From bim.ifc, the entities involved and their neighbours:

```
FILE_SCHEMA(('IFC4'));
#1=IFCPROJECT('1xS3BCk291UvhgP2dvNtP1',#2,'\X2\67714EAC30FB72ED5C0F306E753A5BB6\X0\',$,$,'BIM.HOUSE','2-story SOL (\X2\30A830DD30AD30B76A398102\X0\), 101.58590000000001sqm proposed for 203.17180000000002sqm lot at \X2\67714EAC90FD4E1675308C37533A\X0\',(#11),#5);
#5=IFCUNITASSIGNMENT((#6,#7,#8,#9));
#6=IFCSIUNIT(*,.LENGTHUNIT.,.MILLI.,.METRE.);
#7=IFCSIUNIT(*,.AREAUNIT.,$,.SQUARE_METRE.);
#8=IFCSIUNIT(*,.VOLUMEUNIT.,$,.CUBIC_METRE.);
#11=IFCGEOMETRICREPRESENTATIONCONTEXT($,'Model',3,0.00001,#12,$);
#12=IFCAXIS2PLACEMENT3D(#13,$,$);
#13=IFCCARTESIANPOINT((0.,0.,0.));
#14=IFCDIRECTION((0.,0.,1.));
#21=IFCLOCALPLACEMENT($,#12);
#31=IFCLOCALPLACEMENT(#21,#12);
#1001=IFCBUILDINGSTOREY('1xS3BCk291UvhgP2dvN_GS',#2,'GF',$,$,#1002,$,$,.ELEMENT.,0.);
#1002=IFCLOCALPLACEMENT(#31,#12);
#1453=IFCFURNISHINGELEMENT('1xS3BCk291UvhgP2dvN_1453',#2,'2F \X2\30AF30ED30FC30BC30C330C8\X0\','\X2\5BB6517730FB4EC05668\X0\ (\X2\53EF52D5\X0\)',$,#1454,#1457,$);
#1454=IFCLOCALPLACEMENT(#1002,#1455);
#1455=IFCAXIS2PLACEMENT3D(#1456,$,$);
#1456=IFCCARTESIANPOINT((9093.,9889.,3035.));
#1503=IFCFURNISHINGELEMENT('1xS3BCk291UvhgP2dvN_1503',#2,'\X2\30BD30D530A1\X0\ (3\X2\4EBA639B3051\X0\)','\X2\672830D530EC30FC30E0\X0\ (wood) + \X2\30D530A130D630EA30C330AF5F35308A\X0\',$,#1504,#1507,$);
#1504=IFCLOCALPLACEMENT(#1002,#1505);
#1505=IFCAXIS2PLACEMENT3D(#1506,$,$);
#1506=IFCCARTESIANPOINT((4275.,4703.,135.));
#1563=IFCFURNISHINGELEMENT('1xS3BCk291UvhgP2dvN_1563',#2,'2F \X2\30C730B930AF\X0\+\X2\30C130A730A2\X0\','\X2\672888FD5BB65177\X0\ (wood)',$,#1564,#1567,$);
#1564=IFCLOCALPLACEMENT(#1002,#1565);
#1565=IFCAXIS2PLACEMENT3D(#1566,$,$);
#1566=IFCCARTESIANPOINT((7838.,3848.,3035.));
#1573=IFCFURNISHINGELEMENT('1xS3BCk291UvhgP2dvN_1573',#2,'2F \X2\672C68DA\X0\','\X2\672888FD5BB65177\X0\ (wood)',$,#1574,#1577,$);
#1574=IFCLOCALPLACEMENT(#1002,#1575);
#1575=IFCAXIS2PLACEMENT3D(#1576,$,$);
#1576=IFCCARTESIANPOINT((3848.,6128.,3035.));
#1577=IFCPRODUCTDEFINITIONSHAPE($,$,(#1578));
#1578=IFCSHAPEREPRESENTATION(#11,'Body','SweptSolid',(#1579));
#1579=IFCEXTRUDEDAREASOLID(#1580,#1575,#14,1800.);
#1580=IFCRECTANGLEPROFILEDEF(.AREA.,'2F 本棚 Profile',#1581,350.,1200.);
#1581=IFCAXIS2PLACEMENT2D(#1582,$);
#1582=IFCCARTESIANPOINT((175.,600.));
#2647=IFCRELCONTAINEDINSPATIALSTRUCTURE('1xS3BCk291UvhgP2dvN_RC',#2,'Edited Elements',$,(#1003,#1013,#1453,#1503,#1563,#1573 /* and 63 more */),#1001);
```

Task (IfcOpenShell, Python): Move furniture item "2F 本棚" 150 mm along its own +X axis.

```python
import ifcopenshell
import ifcopenshell.api.geometry
import ifcopenshell.util.placement

model = ifcopenshell.open("bim.ifc")

item = model.by_id(1573)
matrix = ifcopenshell.util.placement.get_local_placement(item.ObjectPlacement)
matrix[:3, 3] += matrix[:3, 0] * 150.0
ifcopenshell.api.geometry.edit_object_placement(model, product=item, matrix=matrix, is_si=False)

print(ifcopenshell.util.placement.get_local_placement(item.ObjectPlacement).round(3) + 0.0)

model.write("bim_rev.ifc")
```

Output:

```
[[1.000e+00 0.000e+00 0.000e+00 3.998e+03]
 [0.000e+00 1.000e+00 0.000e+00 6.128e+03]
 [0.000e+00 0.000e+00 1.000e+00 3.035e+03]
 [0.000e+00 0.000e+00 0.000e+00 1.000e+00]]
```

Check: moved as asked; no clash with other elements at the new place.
